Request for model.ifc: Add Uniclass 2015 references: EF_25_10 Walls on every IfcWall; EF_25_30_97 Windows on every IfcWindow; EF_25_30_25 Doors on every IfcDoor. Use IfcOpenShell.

First a look at what the model holds.

```python
import ifcopenshell

model = ifcopenshell.open("model.ifc")
print(model.schema)
print("classifications:", [c.Name for c in model.by_type("IfcClassification")])
for ifc_class in ("IfcDoor", "IfcRoof", "IfcStair", "IfcWall", "IfcWindow"):
    print(ifc_class, len(model.by_type(ifc_class)))
```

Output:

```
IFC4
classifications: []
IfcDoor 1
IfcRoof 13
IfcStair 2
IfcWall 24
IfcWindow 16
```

```python
import ifcopenshell
import ifcopenshell.api.classification

model = ifcopenshell.open("model.ifc")

system = ifcopenshell.api.classification.add_classification(model, classification="Uniclass 2015")

codes = {
    "IfcWall": ("EF_25_10", "Walls"),
    "IfcWindow": ("EF_25_30_97", "Windows"),
    "IfcDoor": ("EF_25_30_25", "Doors"),
}
for ifc_class, (code, name) in codes.items():
    products = model.by_type(ifc_class)
    ifcopenshell.api.classification.add_reference(
        model, products=products, classification=system, identification=code, name=name
    )
    print(code, len(products))

model.write("model_edited.ifc")
```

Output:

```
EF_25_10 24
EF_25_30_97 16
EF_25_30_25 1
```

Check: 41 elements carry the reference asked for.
